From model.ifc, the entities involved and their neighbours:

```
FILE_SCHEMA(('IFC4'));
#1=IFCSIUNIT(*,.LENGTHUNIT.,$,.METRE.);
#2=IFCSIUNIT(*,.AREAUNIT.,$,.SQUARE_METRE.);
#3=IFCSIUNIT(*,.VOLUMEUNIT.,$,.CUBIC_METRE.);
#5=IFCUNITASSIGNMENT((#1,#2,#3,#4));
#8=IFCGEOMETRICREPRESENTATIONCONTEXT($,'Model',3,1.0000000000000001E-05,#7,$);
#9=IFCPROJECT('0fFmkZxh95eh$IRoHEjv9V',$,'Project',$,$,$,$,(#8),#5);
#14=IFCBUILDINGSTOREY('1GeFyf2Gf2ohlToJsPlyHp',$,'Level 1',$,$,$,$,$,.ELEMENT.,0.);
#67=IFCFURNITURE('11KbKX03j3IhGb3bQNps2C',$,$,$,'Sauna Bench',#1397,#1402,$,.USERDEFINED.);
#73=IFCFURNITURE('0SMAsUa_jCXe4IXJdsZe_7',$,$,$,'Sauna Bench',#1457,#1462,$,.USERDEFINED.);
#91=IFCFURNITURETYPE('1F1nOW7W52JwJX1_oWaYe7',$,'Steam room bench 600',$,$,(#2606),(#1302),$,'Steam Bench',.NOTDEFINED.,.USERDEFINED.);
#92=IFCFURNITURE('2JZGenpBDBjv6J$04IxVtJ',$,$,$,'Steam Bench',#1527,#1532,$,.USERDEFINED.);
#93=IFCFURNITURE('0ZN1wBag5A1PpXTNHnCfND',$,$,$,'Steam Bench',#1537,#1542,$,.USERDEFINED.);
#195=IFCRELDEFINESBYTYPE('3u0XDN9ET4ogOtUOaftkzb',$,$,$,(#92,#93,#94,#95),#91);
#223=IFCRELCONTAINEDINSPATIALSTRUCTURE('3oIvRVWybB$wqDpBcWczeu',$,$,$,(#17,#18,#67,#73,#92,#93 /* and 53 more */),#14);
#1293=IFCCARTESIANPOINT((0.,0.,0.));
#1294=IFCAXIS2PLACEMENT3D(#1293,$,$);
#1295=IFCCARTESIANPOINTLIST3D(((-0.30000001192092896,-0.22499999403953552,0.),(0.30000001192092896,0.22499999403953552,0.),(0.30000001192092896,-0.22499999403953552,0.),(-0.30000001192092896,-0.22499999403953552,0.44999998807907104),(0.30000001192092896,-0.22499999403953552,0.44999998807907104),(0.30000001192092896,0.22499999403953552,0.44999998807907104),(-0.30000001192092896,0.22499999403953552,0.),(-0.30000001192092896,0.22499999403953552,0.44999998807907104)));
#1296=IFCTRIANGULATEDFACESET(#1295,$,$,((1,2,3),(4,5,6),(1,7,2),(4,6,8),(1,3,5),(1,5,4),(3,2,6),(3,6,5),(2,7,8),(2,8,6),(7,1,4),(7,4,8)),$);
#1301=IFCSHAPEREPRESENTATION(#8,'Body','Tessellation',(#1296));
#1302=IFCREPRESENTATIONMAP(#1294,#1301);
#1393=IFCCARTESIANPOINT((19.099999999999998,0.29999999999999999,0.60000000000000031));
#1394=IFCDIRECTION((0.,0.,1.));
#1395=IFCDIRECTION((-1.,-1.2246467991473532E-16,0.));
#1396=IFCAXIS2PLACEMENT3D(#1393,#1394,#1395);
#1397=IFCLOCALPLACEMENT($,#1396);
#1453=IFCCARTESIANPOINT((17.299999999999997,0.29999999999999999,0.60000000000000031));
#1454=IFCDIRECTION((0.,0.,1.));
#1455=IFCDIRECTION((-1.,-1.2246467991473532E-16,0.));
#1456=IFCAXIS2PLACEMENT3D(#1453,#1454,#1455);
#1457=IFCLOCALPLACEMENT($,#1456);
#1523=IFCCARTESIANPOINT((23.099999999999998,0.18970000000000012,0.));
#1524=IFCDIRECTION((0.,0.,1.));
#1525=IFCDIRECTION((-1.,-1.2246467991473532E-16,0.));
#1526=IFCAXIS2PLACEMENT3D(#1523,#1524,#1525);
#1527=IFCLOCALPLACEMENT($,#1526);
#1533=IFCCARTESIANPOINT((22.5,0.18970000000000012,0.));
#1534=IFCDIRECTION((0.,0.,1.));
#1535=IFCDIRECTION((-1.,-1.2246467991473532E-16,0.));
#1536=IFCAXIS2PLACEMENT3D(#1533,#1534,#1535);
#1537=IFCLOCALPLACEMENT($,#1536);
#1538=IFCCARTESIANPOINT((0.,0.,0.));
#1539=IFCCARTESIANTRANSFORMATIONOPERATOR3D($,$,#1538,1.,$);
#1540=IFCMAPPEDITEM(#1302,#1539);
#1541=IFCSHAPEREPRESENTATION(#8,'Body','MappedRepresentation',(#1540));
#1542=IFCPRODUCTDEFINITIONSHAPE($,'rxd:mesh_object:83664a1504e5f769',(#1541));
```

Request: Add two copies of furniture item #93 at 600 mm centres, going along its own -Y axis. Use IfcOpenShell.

```python
import ifcopenshell
import ifcopenshell.api.geometry
import ifcopenshell.api.root
import ifcopenshell.util.element
import ifcopenshell.util.placement

model = ifcopenshell.open("model.ifc")

source = model.by_id(93)
base = ifcopenshell.util.placement.get_local_placement(source.ObjectPlacement)
step = -base[:3, 1] * 0.6

for i in range(1, 3):
    copy = ifcopenshell.api.root.copy_class(model, product=source)
    copy.Representation = ifcopenshell.util.element.copy_deep(
        model, source.Representation, exclude=["IfcGeometricRepresentationContext", "IfcRepresentationMap"]
    )
    matrix = base.copy()
    matrix[:3, 3] += i * step
    print("added at", matrix[:3, 3].round(3) + 0.0)
    ifcopenshell.api.geometry.edit_object_placement(model, product=copy, matrix=matrix, is_si=False)

model.write("model_edited.ifc")
```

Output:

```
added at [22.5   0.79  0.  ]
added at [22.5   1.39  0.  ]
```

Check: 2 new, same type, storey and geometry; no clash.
